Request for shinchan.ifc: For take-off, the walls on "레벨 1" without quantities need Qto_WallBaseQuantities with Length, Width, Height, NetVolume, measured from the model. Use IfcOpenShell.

First a look at what the model holds.

```python
import ifcopenshell
import ifcopenshell.util.element
import ifcopenshell.util.unit

model = ifcopenshell.open("shinchan.ifc")
print(model.schema)
for unit_type in ("LENGTHUNIT", "AREAUNIT", "VOLUMEUNIT"):
    print(unit_type, ifcopenshell.util.unit.calculate_unit_scale(model, unit_type))
storey = next(s for s in model.by_type("IfcBuildingStorey") if s.Name == "레벨 1")
walls = [e for e in ifcopenshell.util.element.get_decomposition(storey) if e.is_a("IfcWall")]
for e in sorted(walls, key=lambda e: e.id()):
    print(e.id(), e.is_a(), e.Name, list(ifcopenshell.util.element.get_psets(e, qtos_only=True)), sep=" | ")
```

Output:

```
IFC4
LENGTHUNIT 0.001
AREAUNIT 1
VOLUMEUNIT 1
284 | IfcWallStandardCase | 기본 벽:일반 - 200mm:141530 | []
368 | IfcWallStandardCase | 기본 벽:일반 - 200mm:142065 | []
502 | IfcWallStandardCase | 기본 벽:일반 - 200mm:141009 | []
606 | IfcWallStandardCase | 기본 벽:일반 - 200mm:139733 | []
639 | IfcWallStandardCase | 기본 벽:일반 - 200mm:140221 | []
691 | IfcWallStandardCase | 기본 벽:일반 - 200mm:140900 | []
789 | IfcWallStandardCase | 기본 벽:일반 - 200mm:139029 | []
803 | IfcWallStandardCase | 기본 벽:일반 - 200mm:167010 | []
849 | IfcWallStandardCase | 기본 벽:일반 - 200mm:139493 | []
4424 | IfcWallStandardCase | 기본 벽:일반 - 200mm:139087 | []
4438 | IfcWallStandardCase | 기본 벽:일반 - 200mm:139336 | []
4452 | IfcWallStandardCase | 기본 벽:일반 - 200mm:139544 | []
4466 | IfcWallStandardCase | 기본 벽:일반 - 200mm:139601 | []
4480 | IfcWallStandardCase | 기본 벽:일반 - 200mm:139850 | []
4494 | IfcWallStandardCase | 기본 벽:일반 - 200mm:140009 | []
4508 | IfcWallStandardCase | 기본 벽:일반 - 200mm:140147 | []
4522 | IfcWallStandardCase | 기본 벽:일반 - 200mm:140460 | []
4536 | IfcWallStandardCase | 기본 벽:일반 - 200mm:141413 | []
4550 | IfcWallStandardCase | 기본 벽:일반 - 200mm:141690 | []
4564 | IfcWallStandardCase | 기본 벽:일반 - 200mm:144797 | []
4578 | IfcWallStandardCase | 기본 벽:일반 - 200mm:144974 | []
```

```python
import ifcopenshell
import ifcopenshell.api.pset
import ifcopenshell.geom
import ifcopenshell.util.element
import ifcopenshell.util.shape
import ifcopenshell.util.unit

model = ifcopenshell.open("shinchan.ifc")
unit_scale = ifcopenshell.util.unit.calculate_unit_scale(model)
volume_scale = ifcopenshell.util.unit.calculate_unit_scale(model, "VOLUMEUNIT")
settings = ifcopenshell.geom.settings()

storey = next(s for s in model.by_type("IfcBuildingStorey") if s.Name == "레벨 1")
walls = [e for e in ifcopenshell.util.element.get_decomposition(storey) if e.is_a("IfcWall")]

for e in sorted(walls, key=lambda e: e.id()):
    if ifcopenshell.util.element.get_psets(e, qtos_only=True, should_inherit=False):
        continue
    # Geometry comes back in metres, in the element's own axes.
    shape = ifcopenshell.geom.create_shape(settings, e)
    values = {
        "Length": ifcopenshell.util.shape.get_x(shape.geometry) / unit_scale,
        "Width": ifcopenshell.util.shape.get_y(shape.geometry) / unit_scale,
        "Height": ifcopenshell.util.shape.get_z(shape.geometry) / unit_scale,
        "NetVolume": ifcopenshell.util.shape.get_volume(shape.geometry) / volume_scale,
    }
    qto = ifcopenshell.api.pset.add_qto(model, product=e, name="Qto_WallBaseQuantities")
    ifcopenshell.api.pset.edit_qto(model, qto=qto, properties=values)
    print(e.id(), {k: round(v, 3) for k, v in values.items()})

model.write("shinchan_updated.ifc")
```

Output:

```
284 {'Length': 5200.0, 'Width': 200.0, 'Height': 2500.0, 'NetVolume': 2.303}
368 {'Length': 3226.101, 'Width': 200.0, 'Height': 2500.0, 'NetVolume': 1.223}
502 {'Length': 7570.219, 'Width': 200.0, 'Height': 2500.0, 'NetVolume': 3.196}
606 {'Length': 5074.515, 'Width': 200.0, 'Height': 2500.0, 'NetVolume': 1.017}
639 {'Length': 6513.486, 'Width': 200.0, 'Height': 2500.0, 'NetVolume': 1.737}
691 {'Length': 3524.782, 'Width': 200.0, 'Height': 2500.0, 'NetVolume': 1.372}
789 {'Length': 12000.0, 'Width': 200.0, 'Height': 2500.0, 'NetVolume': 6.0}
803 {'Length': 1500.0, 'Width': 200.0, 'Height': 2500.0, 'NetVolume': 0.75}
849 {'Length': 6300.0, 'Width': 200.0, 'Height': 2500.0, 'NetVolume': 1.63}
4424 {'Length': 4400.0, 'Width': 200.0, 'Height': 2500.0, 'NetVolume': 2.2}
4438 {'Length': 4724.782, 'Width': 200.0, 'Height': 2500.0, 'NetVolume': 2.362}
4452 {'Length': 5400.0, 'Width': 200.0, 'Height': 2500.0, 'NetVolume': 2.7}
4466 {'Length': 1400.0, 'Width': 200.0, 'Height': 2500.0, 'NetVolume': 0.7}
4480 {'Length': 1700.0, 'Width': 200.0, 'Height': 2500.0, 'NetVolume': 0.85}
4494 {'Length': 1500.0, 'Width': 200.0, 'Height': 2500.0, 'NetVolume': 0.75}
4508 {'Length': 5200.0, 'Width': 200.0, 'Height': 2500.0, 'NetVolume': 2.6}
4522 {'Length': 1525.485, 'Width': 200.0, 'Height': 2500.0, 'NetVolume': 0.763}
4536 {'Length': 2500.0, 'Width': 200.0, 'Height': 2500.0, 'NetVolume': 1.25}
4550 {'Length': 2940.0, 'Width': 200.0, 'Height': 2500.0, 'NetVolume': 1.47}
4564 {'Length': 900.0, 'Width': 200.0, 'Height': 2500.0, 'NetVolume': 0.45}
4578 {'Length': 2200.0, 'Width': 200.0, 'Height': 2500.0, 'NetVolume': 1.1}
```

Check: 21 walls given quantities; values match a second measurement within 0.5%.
